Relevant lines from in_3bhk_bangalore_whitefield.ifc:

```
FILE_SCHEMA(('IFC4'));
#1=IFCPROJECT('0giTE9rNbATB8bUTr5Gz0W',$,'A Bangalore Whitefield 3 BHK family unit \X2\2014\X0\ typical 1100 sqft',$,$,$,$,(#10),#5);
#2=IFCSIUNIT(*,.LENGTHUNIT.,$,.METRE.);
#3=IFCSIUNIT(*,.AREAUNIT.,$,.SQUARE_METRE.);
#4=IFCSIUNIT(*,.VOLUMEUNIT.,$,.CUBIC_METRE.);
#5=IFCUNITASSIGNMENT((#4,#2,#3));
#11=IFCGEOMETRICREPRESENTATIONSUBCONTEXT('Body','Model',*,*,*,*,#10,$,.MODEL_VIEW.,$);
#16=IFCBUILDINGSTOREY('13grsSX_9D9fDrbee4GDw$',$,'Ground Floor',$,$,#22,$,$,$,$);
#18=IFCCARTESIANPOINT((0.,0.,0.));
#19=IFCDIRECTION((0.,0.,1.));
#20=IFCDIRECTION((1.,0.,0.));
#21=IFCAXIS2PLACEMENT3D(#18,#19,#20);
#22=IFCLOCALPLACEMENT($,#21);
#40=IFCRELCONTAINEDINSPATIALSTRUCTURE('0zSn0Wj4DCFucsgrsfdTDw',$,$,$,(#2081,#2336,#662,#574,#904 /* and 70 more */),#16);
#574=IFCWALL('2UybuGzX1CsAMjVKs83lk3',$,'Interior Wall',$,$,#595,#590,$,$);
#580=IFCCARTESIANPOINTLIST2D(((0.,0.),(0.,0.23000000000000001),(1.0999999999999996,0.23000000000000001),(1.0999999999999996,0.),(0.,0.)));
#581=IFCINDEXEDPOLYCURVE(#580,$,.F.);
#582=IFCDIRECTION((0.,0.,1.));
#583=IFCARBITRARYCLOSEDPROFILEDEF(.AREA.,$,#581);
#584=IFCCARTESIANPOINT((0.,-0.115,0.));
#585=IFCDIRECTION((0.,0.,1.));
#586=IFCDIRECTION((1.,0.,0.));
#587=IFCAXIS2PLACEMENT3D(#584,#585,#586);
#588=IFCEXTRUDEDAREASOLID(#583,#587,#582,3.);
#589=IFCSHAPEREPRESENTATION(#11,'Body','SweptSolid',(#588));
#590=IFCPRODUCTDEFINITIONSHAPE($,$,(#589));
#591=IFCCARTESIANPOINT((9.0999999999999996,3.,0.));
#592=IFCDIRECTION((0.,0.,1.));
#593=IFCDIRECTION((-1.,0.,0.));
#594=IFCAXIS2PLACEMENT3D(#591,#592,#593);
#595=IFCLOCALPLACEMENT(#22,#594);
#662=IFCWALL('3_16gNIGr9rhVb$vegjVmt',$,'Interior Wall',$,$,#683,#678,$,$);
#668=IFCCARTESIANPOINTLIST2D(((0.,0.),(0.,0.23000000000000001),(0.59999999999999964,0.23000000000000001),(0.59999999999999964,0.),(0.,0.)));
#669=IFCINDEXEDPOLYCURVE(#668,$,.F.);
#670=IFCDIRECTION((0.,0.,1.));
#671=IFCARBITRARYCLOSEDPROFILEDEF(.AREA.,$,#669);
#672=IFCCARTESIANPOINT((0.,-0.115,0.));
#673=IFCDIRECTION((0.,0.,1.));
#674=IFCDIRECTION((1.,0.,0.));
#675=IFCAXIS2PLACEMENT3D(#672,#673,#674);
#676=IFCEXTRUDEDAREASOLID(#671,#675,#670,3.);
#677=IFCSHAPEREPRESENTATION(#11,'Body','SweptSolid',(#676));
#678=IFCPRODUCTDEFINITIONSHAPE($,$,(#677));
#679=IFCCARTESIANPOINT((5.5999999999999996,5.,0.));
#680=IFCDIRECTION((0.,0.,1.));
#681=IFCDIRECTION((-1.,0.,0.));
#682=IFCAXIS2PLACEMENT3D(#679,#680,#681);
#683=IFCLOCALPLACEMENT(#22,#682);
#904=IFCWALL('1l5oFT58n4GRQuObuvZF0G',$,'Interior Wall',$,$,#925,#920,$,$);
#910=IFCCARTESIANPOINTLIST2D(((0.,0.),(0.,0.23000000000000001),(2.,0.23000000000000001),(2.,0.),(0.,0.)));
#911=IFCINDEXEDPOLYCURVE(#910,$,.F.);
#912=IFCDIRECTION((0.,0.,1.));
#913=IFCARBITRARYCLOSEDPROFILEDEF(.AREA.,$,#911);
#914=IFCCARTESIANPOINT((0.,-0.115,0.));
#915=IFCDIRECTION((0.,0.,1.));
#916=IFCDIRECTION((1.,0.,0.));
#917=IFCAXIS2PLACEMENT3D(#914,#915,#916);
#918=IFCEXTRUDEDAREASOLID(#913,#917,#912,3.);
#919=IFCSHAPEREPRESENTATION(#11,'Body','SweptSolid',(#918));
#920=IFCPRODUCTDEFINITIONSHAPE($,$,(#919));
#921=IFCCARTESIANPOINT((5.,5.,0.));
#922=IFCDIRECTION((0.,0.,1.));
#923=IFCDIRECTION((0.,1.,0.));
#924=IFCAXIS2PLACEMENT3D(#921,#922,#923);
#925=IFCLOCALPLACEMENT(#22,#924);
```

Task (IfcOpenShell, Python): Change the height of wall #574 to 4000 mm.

```python
import ifcopenshell
import ifcopenshell.geom
import ifcopenshell.util.representation
import ifcopenshell.util.shape
import ifcopenshell.util.unit

model = ifcopenshell.open("in_3bhk_bangalore_whitefield.ifc")
unit_scale = ifcopenshell.util.unit.calculate_unit_scale(model)
settings = ifcopenshell.geom.settings()


def volume(element):
    """Net volume in cubic metres, openings subtracted."""
    shape = ifcopenshell.geom.create_shape(settings, element)
    return ifcopenshell.util.shape.get_volume(shape.geometry)


wall = model.by_id(574)
before = volume(wall)

body = ifcopenshell.util.representation.get_representation(wall, "Model", "Body")
solid = body.Items[0]
old_height = solid.Depth
solid.Depth = 4 / unit_scale
after = volume(wall)

print(f"height {old_height:g} -> {solid.Depth:g}, volume {before:.3f} -> {after:.3f} m3")

model.write("in_3bhk_bangalore_whitefield_updated.ifc")
```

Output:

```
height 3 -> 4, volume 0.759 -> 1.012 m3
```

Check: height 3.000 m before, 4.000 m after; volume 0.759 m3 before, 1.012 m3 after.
